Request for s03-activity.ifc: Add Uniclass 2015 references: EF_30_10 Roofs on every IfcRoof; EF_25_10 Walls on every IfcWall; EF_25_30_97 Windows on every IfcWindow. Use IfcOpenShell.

First a look at what the model holds.

```python
import ifcopenshell

model = ifcopenshell.open("s03-activity.ifc")
print(model.schema)
print("classifications:", [c.Name for c in model.by_type("IfcClassification")])
for ifc_class in ("IfcDoor", "IfcRoof", "IfcStair", "IfcWall", "IfcWindow"):
    print(ifc_class, len(model.by_type(ifc_class)))
```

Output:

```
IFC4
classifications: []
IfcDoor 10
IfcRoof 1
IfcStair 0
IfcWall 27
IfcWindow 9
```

```python
import ifcopenshell
import ifcopenshell.api.classification

model = ifcopenshell.open("s03-activity.ifc")

system = ifcopenshell.api.classification.add_classification(model, classification="Uniclass 2015")

codes = {
    "IfcRoof": ("EF_30_10", "Roofs"),
    "IfcWall": ("EF_25_10", "Walls"),
    "IfcWindow": ("EF_25_30_97", "Windows"),
}
for ifc_class, (code, name) in codes.items():
    products = model.by_type(ifc_class)
    ifcopenshell.api.classification.add_reference(
        model, products=products, classification=system, identification=code, name=name
    )
    print(code, len(products))

model.write("s03-activity_edited.ifc")
```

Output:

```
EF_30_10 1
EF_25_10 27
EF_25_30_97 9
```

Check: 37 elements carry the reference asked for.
